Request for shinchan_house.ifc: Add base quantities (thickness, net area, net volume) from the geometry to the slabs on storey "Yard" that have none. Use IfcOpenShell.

First a look at what the model holds.

```python
import ifcopenshell
import ifcopenshell.util.element
import ifcopenshell.util.unit

model = ifcopenshell.open("shinchan_house.ifc")
print(model.schema)
for unit_type in ("LENGTHUNIT", "AREAUNIT", "VOLUMEUNIT"):
    print(unit_type, ifcopenshell.util.unit.calculate_unit_scale(model, unit_type))
storey = next(s for s in model.by_type("IfcBuildingStorey") if s.Name == "Yard")
slabs = [e for e in ifcopenshell.util.element.get_decomposition(storey) if e.is_a("IfcSlab")]
for e in sorted(slabs, key=lambda e: e.id()):
    print(e.id(), e.is_a(), e.Name, list(ifcopenshell.util.element.get_psets(e, qtos_only=True)), sep=" | ")
```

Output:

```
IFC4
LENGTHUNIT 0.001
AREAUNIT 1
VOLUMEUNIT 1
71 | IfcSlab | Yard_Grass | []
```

```python
import ifcopenshell
import ifcopenshell.api.pset
import ifcopenshell.geom
import ifcopenshell.util.element
import ifcopenshell.util.shape
import ifcopenshell.util.unit

model = ifcopenshell.open("shinchan_house.ifc")
unit_scale = ifcopenshell.util.unit.calculate_unit_scale(model)
area_scale = ifcopenshell.util.unit.calculate_unit_scale(model, "AREAUNIT")
volume_scale = ifcopenshell.util.unit.calculate_unit_scale(model, "VOLUMEUNIT")
settings = ifcopenshell.geom.settings()

storey = next(s for s in model.by_type("IfcBuildingStorey") if s.Name == "Yard")
slabs = [e for e in ifcopenshell.util.element.get_decomposition(storey) if e.is_a("IfcSlab")]

for e in sorted(slabs, key=lambda e: e.id()):
    if ifcopenshell.util.element.get_psets(e, qtos_only=True, should_inherit=False):
        continue
    # Geometry comes back in metres, in the element's own axes.
    shape = ifcopenshell.geom.create_shape(settings, e)
    values = {
        "Width": ifcopenshell.util.shape.get_z(shape.geometry) / unit_scale,
        "NetArea": ifcopenshell.util.shape.get_footprint_area(shape.geometry) / area_scale,
        "NetVolume": ifcopenshell.util.shape.get_volume(shape.geometry) / volume_scale,
    }
    qto = ifcopenshell.api.pset.add_qto(model, product=e, name="Qto_SlabBaseQuantities")
    ifcopenshell.api.pset.edit_qto(model, qto=qto, properties=values)
    print(e.id(), {k: round(v, 3) for k, v in values.items()})

model.write("shinchan_house_rev.ifc")
```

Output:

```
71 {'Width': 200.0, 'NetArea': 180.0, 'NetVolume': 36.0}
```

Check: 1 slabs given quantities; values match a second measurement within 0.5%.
